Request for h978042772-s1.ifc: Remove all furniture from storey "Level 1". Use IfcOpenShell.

First a look at what the model holds.

```python
import ifcopenshell
import ifcopenshell.util.element

model = ifcopenshell.open("h978042772-s1.ifc")
print(model.schema)
storey = next(s for s in model.by_type("IfcBuildingStorey") if s.Name == "Level 1")
furniture = [e for e in ifcopenshell.util.element.get_decomposition(storey) if e.is_a("IfcFurnishingElement")]
seen = {}
for e in furniture:
    element_type = ifcopenshell.util.element.get_type(e)
    name = element_type.Name if element_type not in (None, e) else None
    seen[name] = seen.get(name, 0) + 1
for name, count in sorted(seen.items(), key=str):
    print(count, "x", name)
```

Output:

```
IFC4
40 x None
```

```python
import ifcopenshell
import ifcopenshell.api.root
import ifcopenshell.util.element

model = ifcopenshell.open("h978042772-s1.ifc")

storey = next(s for s in model.by_type("IfcBuildingStorey") if s.Name == "Level 1")
furniture = [e for e in ifcopenshell.util.element.get_decomposition(storey) if e.is_a("IfcFurnishingElement")]

for e in furniture:
    ifcopenshell.api.root.remove_product(model, product=e)
print(len(furniture), "removed")

model.write("h978042772-s1-out.ifc")
```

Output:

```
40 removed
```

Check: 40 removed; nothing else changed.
